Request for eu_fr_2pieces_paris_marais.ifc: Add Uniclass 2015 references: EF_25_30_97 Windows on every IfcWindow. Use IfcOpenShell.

First a look at what the model holds.

```python
import ifcopenshell

model = ifcopenshell.open("eu_fr_2pieces_paris_marais.ifc")
print(model.schema)
print("classifications:", [c.Name for c in model.by_type("IfcClassification")])
for ifc_class in ("IfcDoor", "IfcRoof", "IfcStair", "IfcWall", "IfcWindow"):
    print(ifc_class, len(model.by_type(ifc_class)))
```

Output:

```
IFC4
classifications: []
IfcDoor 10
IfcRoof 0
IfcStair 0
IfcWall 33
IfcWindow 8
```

```python
import ifcopenshell
import ifcopenshell.api.classification

model = ifcopenshell.open("eu_fr_2pieces_paris_marais.ifc")

system = ifcopenshell.api.classification.add_classification(model, classification="Uniclass 2015")

codes = {
    "IfcWindow": ("EF_25_30_97", "Windows"),
}
for ifc_class, (code, name) in codes.items():
    products = model.by_type(ifc_class)
    ifcopenshell.api.classification.add_reference(
        model, products=products, classification=system, identification=code, name=name
    )
    print(code, len(products))

model.write("eu_fr_2pieces_paris_marais_updated.ifc")
```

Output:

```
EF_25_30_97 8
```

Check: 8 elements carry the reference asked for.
